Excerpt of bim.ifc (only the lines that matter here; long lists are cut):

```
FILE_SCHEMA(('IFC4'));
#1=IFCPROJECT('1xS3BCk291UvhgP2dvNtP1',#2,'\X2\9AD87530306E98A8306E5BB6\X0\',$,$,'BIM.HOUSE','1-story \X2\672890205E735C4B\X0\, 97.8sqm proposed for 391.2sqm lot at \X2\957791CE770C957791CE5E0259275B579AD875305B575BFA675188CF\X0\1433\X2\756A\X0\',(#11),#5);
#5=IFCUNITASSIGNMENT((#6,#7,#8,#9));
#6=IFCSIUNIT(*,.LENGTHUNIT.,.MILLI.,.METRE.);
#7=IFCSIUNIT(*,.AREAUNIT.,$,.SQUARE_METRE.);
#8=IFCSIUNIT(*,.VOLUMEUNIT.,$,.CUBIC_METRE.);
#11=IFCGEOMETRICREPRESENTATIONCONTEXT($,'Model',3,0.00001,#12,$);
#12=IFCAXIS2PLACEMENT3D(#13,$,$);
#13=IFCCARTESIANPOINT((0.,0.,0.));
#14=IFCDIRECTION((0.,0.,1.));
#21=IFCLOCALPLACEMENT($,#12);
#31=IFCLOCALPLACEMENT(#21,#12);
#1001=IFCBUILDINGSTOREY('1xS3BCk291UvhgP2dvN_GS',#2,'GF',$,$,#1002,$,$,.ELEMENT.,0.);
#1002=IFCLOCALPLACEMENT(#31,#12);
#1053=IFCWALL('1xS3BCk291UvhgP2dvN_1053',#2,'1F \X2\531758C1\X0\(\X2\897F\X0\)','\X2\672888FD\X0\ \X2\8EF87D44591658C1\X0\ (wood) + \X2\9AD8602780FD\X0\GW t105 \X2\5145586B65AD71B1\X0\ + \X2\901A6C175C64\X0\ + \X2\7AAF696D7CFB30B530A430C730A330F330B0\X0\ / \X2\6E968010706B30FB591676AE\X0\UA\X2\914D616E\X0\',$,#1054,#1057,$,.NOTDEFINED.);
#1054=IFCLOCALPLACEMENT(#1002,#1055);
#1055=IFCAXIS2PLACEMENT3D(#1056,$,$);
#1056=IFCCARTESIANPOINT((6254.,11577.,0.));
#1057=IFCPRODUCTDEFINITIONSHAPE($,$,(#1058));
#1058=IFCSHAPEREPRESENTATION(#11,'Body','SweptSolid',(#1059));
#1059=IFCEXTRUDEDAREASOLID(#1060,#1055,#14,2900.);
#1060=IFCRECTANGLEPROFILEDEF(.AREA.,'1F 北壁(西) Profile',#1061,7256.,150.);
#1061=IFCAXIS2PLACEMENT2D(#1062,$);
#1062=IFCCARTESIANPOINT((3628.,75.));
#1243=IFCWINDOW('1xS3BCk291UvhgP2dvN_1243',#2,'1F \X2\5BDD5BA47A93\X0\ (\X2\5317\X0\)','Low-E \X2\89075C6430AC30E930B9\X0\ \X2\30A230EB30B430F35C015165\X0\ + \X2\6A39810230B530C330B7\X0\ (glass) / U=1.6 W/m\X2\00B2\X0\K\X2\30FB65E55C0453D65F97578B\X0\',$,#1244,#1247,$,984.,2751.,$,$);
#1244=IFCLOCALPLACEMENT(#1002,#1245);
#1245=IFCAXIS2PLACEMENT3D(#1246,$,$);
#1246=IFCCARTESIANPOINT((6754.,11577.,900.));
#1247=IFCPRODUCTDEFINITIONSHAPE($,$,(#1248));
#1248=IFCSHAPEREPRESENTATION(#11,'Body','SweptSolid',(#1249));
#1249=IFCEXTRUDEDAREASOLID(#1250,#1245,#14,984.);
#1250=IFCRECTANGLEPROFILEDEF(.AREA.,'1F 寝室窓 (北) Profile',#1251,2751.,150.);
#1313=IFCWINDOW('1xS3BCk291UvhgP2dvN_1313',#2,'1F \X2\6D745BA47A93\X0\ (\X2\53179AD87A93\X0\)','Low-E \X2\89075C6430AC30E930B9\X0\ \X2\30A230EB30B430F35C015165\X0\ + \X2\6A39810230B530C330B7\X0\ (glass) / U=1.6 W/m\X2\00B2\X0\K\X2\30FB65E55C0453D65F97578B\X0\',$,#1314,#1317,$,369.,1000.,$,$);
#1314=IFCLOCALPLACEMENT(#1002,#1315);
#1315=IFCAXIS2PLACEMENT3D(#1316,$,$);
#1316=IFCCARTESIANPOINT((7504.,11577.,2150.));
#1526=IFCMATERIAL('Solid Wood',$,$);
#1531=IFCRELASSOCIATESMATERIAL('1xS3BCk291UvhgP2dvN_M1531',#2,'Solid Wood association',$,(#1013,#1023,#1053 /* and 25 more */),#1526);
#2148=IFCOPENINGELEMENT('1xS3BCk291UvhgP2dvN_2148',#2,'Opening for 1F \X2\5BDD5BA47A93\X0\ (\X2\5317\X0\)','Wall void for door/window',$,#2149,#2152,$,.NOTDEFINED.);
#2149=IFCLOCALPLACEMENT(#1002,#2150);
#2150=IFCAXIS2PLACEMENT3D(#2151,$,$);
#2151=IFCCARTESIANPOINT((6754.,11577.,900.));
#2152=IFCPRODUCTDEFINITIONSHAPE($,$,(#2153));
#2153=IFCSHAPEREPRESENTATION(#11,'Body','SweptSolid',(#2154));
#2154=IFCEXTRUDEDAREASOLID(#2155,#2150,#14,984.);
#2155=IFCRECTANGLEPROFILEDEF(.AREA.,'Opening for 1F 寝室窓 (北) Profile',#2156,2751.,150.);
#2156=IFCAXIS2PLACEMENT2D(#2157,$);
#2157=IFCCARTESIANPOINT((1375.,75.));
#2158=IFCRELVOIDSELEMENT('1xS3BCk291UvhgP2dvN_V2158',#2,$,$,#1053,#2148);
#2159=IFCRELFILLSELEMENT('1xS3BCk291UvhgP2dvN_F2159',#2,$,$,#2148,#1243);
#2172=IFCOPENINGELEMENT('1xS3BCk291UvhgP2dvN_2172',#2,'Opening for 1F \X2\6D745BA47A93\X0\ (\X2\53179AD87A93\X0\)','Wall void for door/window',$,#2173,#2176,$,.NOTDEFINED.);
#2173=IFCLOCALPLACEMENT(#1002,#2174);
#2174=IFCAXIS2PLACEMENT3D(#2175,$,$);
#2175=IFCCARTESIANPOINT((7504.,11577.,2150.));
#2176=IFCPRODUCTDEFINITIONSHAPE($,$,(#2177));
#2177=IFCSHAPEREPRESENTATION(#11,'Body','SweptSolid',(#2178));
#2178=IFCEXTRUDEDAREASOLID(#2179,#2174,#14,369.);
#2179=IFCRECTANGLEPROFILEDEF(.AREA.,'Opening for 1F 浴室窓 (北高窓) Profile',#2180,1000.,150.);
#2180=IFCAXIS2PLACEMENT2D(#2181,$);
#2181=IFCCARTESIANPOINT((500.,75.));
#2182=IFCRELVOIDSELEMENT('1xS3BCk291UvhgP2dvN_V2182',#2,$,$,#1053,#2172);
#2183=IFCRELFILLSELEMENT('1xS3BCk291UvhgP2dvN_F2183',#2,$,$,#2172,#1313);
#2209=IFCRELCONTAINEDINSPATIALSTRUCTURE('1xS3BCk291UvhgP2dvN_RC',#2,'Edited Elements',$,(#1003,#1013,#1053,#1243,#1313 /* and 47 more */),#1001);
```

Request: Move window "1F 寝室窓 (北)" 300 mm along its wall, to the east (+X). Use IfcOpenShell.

```python
import ifcopenshell
import ifcopenshell.api.geometry
import ifcopenshell.util.placement

model = ifcopenshell.open("bim.ifc")

window = model.by_id(1243)
opening = window.FillsVoids[0].RelatingOpeningElement
wall = opening.VoidsElements[0].RelatingBuildingElement

wall_matrix = ifcopenshell.util.placement.get_local_placement(wall.ObjectPlacement)
shift = wall_matrix[:3, 0] * 300.0
before = ifcopenshell.util.placement.get_local_placement(window.ObjectPlacement)[:3, 3].copy()

# The window is not placed relative to its opening, so move both.
for product in (opening, window):
    matrix = ifcopenshell.util.placement.get_local_placement(product.ObjectPlacement)
    matrix[:3, 3] += shift
    ifcopenshell.api.geometry.edit_object_placement(model, product=product, matrix=matrix, is_si=False)

after = ifcopenshell.util.placement.get_local_placement(window.ObjectPlacement)[:3, 3]
print("window moved by", (after - before).round(3) + 0.0)

model.write("bim_updated.ifc")
```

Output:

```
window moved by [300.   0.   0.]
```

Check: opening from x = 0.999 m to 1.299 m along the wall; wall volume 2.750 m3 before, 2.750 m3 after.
